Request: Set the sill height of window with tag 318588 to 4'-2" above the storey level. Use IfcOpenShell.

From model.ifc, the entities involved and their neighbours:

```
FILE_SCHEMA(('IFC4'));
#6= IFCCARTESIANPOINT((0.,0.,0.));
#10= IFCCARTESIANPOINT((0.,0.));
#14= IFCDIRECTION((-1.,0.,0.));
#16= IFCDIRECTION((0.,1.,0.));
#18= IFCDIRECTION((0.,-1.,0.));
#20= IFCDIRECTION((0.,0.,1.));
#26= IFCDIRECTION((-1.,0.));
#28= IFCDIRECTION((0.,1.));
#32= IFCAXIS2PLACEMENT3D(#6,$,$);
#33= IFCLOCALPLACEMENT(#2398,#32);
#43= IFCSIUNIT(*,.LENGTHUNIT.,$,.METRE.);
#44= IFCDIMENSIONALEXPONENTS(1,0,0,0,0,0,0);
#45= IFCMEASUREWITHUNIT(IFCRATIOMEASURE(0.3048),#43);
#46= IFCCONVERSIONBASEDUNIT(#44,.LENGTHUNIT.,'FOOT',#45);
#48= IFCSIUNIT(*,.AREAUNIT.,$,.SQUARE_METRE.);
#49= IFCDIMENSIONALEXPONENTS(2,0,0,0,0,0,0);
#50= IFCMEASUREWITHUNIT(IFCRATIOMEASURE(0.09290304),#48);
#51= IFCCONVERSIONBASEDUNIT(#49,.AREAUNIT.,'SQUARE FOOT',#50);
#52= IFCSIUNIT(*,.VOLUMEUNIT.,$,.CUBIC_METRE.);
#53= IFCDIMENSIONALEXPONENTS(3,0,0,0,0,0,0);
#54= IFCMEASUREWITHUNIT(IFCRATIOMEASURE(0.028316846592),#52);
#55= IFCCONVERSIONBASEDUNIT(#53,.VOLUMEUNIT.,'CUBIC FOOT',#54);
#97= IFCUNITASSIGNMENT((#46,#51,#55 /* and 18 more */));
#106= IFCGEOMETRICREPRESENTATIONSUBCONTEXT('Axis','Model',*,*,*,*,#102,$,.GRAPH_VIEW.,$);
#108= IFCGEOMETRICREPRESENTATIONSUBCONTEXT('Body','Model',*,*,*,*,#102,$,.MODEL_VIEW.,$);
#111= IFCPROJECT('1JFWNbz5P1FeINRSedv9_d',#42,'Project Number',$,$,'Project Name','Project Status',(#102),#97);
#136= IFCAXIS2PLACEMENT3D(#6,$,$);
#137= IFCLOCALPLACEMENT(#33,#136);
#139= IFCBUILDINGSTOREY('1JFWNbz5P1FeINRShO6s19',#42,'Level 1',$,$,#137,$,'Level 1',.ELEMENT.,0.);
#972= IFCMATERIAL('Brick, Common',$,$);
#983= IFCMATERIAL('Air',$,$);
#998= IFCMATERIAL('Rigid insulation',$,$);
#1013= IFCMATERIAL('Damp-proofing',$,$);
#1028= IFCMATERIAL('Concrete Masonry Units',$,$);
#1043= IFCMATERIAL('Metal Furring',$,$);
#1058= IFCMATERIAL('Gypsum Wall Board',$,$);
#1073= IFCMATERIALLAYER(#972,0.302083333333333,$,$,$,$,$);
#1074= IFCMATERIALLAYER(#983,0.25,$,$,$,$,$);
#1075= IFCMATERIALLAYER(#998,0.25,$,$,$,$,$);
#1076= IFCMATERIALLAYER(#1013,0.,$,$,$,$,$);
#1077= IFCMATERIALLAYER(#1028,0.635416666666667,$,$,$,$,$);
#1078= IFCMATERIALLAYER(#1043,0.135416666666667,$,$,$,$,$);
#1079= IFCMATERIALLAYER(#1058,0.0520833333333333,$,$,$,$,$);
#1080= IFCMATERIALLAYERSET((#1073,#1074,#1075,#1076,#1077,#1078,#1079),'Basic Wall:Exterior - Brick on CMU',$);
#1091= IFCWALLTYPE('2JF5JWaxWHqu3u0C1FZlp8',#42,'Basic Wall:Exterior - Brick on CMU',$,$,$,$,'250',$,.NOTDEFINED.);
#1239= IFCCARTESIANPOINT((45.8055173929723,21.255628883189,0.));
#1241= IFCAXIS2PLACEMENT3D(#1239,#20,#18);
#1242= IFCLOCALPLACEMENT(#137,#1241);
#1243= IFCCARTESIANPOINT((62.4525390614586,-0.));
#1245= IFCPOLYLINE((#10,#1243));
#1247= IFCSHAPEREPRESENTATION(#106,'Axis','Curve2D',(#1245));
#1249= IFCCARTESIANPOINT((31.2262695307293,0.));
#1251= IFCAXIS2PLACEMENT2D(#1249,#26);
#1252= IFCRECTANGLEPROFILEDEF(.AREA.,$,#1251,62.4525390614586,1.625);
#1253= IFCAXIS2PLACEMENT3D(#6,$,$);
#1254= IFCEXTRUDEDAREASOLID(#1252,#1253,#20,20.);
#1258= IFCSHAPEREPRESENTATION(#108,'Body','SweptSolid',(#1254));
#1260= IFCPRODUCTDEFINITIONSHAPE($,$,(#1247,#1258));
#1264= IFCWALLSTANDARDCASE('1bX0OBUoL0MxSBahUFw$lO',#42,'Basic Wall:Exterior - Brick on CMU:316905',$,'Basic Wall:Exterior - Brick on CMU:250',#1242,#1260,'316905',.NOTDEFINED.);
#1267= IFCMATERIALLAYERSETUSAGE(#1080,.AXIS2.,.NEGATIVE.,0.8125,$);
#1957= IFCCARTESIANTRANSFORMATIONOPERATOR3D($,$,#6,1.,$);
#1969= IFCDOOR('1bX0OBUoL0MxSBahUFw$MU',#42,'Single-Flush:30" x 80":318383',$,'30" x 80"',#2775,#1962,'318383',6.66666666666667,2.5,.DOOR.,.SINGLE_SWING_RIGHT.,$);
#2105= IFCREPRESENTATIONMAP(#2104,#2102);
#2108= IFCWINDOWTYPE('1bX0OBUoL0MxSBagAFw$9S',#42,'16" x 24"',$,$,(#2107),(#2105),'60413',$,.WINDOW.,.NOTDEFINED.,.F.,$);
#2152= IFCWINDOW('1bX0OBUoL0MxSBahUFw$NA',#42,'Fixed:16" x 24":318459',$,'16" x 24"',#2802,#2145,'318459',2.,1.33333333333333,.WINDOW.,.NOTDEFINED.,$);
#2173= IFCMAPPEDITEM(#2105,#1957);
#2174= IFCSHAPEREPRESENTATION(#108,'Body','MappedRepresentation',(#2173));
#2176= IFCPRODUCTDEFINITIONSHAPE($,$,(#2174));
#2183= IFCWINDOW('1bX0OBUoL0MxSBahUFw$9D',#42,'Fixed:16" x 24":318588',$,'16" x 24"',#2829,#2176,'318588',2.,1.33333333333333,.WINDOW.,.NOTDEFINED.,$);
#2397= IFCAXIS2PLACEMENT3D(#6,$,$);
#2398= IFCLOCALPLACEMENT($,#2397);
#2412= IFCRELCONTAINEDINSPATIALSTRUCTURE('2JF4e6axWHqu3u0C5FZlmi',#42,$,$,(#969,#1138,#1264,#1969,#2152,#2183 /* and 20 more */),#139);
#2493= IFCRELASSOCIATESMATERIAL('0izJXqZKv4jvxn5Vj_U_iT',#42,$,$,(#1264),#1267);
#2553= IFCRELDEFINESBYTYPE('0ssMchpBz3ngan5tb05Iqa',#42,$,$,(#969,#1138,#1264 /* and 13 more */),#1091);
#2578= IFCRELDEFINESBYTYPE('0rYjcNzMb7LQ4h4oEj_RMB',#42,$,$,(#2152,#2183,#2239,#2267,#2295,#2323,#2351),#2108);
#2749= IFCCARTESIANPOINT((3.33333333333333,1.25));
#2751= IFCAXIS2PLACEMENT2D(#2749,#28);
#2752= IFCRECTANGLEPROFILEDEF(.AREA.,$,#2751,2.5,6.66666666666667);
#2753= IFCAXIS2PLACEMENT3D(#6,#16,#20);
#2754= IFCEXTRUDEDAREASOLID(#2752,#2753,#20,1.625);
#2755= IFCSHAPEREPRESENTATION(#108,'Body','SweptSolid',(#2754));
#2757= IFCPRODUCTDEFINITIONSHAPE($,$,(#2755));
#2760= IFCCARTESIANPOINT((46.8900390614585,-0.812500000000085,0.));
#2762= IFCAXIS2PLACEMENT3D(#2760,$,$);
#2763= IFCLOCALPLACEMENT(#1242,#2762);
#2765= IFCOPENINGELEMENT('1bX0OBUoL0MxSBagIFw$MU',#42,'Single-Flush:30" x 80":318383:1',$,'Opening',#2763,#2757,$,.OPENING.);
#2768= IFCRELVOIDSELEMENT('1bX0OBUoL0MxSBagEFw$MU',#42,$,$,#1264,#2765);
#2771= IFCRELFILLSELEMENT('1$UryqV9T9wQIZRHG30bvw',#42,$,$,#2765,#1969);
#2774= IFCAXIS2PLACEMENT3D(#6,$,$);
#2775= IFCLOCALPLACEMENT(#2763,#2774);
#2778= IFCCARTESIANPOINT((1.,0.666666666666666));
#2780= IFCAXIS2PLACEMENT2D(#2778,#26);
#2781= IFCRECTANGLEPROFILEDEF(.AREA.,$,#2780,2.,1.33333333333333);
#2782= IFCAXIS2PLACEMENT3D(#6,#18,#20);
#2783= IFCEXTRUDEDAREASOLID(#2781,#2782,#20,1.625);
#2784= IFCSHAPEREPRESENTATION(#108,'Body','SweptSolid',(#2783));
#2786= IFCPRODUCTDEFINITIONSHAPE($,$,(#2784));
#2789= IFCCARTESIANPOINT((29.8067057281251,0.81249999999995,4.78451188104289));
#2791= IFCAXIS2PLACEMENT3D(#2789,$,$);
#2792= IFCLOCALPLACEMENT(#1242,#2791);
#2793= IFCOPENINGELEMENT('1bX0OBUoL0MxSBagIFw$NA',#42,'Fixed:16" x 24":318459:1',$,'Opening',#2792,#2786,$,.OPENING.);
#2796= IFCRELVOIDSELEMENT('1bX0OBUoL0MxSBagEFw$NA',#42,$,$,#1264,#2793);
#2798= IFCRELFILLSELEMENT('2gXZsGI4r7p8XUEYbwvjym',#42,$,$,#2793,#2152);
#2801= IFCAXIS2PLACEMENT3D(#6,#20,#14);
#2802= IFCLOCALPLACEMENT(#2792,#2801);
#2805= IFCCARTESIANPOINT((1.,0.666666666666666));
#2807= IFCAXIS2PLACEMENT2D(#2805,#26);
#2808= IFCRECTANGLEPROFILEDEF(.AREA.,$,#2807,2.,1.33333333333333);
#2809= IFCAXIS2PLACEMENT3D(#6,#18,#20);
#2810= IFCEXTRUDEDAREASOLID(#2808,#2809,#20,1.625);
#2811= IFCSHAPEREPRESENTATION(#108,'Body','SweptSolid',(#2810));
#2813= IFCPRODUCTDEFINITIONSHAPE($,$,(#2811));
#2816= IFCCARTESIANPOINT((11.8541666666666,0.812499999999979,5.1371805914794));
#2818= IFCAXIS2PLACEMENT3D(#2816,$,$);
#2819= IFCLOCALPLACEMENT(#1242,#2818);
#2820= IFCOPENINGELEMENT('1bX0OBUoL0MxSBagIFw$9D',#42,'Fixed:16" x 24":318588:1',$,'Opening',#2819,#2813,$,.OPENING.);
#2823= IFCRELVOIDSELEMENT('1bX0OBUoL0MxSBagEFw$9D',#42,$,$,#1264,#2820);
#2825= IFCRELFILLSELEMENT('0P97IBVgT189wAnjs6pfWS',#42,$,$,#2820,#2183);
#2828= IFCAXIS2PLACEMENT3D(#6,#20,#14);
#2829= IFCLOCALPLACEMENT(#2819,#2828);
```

```python
import numpy as np
import ifcopenshell
import ifcopenshell.api.geometry
import ifcopenshell.geom
import ifcopenshell.util.element
import ifcopenshell.util.placement
import ifcopenshell.util.shape
import ifcopenshell.util.unit

model = ifcopenshell.open("model.ifc")
unit_scale = ifcopenshell.util.unit.calculate_unit_scale(model)

window = model.by_guid("1bX0OBUoL0MxSBahUFw$9D")
opening = window.FillsVoids[0].RelatingOpeningElement
storey = ifcopenshell.util.element.get_container(window, ifc_class="IfcBuildingStorey")
level = ifcopenshell.util.placement.get_local_placement(storey.ObjectPlacement)[2, 3]

# The opening's origin need not be at the sill, so measure its lowest point.
shape = ifcopenshell.geom.create_shape(ifcopenshell.geom.settings(), opening)
bottom = ifcopenshell.util.shape.get_shape_bottom_elevation(shape, shape.geometry) / unit_scale
dz = level + 50 * 0.0254 / unit_scale - bottom

shift = np.array([0.0, 0.0, dz])
# The window is placed relative to its opening, so it follows when the opening moves.
matrix = ifcopenshell.util.placement.get_local_placement(opening.ObjectPlacement)
matrix[:3, 3] += shift
ifcopenshell.api.geometry.edit_object_placement(
    model, product=opening, matrix=matrix, is_si=False, should_transform_children=True
)

print(f"moved by {dz * unit_scale:+.3f} m")

model.write("model_v2.ifc")
```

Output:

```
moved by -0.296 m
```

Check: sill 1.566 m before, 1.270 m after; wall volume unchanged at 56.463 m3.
